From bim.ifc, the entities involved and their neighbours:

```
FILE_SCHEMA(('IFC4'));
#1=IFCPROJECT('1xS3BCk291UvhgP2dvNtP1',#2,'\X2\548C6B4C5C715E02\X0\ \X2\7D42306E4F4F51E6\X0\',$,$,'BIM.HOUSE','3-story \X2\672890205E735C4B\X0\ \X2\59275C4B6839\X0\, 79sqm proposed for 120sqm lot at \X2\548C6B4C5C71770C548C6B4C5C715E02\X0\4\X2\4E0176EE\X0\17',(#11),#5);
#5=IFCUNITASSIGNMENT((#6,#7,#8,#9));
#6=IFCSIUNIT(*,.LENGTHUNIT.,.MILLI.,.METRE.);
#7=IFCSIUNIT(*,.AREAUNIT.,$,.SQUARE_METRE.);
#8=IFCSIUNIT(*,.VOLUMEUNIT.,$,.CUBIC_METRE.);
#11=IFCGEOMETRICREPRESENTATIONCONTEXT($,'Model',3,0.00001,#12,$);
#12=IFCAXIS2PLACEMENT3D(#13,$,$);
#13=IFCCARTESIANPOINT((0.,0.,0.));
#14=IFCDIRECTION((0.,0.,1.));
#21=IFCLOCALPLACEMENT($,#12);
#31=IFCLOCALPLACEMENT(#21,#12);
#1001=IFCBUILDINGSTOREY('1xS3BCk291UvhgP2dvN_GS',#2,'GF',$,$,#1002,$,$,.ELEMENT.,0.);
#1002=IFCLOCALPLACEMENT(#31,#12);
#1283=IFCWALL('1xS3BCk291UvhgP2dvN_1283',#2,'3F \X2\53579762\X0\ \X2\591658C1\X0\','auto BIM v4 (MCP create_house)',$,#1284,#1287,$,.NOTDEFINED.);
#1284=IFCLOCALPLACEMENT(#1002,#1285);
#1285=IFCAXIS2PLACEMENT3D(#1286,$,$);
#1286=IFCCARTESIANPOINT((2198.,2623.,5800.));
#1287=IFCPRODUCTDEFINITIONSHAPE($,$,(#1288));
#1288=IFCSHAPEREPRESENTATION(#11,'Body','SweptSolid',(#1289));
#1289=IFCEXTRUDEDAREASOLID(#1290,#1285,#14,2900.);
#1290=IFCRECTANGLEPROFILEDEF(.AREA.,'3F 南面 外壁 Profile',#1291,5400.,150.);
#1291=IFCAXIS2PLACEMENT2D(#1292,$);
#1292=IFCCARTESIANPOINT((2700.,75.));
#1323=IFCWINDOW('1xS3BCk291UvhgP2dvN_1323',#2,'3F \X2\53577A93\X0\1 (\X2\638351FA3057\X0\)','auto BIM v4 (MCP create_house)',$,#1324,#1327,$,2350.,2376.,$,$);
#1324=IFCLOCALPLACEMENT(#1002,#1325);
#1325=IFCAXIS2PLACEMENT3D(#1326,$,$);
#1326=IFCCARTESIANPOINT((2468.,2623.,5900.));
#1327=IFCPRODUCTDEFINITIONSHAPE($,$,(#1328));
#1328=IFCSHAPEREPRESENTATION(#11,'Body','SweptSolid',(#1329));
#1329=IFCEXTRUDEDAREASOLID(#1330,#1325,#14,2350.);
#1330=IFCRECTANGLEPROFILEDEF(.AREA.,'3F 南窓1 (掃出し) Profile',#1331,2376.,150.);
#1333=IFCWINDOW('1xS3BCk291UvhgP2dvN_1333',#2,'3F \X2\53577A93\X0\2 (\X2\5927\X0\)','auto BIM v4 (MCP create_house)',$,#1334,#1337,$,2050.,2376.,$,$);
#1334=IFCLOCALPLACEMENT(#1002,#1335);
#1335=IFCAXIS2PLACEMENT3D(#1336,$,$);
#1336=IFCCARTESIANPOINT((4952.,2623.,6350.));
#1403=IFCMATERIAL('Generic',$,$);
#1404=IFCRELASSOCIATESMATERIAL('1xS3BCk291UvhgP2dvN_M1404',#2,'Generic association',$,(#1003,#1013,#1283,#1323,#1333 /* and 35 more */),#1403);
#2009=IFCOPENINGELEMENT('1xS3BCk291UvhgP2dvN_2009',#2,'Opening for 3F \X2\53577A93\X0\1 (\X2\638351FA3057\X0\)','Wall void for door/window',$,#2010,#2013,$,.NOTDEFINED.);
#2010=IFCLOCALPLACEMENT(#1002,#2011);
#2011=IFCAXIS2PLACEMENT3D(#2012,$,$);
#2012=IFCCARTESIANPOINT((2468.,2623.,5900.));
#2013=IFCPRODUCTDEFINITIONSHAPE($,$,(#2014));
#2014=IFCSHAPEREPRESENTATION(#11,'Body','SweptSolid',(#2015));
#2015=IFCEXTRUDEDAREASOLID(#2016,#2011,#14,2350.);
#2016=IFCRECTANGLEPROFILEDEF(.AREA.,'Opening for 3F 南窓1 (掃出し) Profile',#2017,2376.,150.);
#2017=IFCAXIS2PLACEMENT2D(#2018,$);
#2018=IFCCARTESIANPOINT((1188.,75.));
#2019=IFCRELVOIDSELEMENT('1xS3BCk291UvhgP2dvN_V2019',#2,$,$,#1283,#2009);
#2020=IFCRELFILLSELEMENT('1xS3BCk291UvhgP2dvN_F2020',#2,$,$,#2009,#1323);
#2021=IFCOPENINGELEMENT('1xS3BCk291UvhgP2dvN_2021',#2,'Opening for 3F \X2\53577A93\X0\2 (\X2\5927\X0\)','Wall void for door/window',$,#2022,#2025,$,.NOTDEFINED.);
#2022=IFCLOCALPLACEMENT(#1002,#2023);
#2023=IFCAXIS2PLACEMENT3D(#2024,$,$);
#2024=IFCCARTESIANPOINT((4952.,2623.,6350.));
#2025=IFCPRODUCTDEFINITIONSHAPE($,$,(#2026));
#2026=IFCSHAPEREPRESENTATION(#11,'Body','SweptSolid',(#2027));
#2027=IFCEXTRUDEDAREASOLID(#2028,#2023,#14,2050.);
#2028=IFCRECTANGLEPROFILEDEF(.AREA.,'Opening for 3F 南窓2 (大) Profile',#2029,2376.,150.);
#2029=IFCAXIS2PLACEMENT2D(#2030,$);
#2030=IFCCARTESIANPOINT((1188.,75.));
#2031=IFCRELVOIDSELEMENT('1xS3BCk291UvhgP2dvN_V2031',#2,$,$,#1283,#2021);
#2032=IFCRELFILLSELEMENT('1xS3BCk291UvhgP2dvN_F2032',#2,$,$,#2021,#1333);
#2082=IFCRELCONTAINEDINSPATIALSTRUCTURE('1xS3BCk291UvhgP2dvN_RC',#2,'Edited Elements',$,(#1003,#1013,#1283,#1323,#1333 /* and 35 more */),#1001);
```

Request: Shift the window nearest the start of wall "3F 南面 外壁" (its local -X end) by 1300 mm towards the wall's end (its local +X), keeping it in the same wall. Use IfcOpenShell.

```python
import ifcopenshell
import ifcopenshell.api.geometry
import ifcopenshell.util.placement
import ifcopenshell.util.unit

model = ifcopenshell.open("bim.ifc")
unit_scale = ifcopenshell.util.unit.calculate_unit_scale(model)

window = model.by_guid("1xS3BCk291UvhgP2dvN_1323")
opening = window.FillsVoids[0].RelatingOpeningElement
wall = opening.VoidsElements[0].RelatingBuildingElement

wall_matrix = ifcopenshell.util.placement.get_local_placement(wall.ObjectPlacement)
shift = wall_matrix[:3, 0] * 1.3 / unit_scale
before = ifcopenshell.util.placement.get_local_placement(window.ObjectPlacement)[:3, 3].copy()

# The window is not placed relative to its opening, so move both.
for product in (opening, window):
    matrix = ifcopenshell.util.placement.get_local_placement(product.ObjectPlacement)
    matrix[:3, 3] += shift
    ifcopenshell.api.geometry.edit_object_placement(model, product=product, matrix=matrix, is_si=False)

after = ifcopenshell.util.placement.get_local_placement(window.ObjectPlacement)[:3, 3]
print("window moved by", (after - before).round(3) + 0.0)

model.write("bim_edited.ifc")
```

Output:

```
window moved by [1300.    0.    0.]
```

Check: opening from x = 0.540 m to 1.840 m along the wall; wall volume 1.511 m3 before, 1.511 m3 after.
